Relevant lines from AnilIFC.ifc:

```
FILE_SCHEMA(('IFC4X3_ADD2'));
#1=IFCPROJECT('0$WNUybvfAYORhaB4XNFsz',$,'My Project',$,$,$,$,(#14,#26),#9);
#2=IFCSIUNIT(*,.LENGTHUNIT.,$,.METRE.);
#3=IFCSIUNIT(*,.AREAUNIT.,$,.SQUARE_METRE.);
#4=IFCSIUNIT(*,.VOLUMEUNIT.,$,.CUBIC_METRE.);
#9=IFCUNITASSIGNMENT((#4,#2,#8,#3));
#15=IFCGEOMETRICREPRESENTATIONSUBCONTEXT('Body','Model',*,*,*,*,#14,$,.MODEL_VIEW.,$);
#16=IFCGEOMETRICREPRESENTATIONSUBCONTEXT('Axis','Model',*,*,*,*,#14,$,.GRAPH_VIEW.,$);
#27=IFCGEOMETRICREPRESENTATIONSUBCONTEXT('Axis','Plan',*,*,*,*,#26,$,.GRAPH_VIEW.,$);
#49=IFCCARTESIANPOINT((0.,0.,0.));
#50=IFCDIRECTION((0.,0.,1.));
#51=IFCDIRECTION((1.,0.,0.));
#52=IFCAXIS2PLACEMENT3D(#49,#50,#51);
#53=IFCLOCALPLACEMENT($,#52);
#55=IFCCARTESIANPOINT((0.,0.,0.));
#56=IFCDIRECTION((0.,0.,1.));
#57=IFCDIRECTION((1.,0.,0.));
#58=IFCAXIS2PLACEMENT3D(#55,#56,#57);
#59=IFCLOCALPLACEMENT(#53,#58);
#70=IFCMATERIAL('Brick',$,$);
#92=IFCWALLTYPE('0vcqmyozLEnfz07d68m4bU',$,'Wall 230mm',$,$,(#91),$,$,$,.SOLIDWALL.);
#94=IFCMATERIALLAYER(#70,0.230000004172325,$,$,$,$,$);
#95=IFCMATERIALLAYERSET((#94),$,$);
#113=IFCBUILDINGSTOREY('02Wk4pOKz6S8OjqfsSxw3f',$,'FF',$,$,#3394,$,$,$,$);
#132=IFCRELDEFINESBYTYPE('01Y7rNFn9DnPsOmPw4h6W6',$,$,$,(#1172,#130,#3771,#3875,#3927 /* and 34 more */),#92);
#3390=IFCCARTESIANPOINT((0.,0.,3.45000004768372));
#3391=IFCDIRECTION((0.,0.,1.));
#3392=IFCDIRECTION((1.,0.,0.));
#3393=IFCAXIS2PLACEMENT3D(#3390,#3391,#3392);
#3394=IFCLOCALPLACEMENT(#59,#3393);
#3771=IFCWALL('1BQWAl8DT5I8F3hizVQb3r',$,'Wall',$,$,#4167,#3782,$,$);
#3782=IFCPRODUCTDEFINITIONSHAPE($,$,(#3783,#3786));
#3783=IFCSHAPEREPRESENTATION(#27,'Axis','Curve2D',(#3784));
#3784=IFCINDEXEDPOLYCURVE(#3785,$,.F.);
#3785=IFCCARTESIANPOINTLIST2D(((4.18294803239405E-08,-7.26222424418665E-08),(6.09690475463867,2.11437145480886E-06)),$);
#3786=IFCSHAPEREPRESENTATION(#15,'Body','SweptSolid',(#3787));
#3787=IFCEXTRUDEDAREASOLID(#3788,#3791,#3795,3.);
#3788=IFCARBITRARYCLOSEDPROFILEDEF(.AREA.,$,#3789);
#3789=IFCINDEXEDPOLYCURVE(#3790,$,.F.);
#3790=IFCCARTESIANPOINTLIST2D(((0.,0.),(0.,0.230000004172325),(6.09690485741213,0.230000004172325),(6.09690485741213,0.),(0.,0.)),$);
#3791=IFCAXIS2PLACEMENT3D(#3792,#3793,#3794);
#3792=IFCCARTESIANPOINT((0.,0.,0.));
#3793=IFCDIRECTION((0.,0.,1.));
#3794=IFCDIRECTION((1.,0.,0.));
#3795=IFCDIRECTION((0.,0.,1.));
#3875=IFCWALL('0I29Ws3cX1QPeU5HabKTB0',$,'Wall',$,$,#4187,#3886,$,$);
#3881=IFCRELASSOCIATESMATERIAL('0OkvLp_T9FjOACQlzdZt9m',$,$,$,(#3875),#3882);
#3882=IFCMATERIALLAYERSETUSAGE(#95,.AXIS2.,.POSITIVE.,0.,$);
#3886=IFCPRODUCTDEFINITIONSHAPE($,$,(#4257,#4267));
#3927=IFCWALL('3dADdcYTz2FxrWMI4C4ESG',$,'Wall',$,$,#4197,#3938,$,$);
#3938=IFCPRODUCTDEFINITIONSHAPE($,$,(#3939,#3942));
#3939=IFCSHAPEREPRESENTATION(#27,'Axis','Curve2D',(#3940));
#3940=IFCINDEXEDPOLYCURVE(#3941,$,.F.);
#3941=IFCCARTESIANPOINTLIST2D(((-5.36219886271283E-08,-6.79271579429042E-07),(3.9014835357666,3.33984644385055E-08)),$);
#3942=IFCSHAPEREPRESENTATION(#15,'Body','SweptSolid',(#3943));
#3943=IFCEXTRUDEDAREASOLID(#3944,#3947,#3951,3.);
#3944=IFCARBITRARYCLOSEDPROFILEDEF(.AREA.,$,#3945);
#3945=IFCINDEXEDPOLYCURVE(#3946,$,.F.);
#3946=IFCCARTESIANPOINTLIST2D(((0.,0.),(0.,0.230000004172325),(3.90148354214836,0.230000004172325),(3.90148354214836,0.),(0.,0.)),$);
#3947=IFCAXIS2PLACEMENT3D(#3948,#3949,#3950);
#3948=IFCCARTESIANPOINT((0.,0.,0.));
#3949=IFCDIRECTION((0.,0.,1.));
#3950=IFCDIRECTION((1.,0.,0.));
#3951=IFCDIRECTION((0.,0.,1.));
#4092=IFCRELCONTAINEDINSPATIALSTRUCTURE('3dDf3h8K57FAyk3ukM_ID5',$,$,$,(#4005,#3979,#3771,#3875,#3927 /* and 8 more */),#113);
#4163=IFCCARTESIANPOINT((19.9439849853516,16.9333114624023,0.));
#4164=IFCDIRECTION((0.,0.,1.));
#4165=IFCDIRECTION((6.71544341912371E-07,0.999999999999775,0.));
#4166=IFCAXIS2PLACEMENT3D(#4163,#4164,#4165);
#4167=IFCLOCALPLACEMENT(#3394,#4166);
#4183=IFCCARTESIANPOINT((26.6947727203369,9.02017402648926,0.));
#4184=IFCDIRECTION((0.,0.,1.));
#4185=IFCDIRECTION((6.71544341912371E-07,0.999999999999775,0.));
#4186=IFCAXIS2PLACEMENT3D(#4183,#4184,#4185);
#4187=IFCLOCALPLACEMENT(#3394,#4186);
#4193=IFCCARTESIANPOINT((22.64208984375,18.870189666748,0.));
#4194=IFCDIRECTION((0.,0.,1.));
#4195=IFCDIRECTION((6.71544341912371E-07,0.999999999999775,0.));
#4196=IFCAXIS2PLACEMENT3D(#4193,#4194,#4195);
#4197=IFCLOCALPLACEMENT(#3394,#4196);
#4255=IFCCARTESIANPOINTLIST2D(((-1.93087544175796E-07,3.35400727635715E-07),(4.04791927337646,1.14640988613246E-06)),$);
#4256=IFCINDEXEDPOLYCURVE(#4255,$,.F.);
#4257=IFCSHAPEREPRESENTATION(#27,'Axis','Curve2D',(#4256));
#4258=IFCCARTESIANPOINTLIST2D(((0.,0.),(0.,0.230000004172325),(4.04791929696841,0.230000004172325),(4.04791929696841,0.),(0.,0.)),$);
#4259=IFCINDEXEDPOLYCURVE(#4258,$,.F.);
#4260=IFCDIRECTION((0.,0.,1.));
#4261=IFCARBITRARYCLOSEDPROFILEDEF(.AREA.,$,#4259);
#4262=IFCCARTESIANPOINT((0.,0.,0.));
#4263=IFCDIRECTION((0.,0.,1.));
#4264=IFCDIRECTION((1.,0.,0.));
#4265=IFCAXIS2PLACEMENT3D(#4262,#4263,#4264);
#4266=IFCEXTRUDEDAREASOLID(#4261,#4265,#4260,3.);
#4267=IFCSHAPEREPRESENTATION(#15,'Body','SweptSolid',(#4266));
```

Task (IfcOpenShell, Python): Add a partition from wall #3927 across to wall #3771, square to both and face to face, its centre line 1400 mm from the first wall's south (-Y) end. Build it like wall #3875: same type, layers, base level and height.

```python
import numpy as np
import ifcopenshell
import ifcopenshell.api.geometry
import ifcopenshell.api.material
import ifcopenshell.api.pset
import ifcopenshell.api.root
import ifcopenshell.api.spatial
import ifcopenshell.api.type
import ifcopenshell.geom
import ifcopenshell.util.element
import ifcopenshell.util.placement
import ifcopenshell.util.representation
import ifcopenshell.util.shape
import ifcopenshell.util.unit

model = ifcopenshell.open("AnilIFC.ifc")
unit_scale = ifcopenshell.util.unit.calculate_unit_scale(model)
settings = ifcopenshell.geom.settings()
settings.set("use-world-coords", True)

start_wall = model.by_guid("3dADdcYTz2FxrWMI4C4ESG")
end_wall = model.by_guid("1BQWAl8DT5I8F3hizVQb3r")
like = model.by_id(3875)
matrix = ifcopenshell.util.placement.get_local_placement(start_wall.ObjectPlacement)
matrix[:3, 3] *= unit_scale


def extent(element):
    """Bounding box in the first wall's axes, in metres."""
    shape = ifcopenshell.geom.create_shape(settings, element)
    points = (ifcopenshell.util.shape.get_vertices(shape.geometry) - matrix[:3, 3]) @ matrix[:3, :3]
    return points.min(axis=0), points.max(axis=0)


y_start = extent(start_wall)[1][1]
y_end = extent(end_wall)[0][1]
like_min, like_max = extent(like)
length, height = float(abs(y_end - y_start)), float(like_max[2] - like_min[2])
layer_set = ifcopenshell.util.element.get_material(like, should_skip_usage=True)
thickness = sum(layer.LayerThickness for layer in layer_set.MaterialLayers) * unit_scale

wall = ifcopenshell.api.root.create_entity(model, ifc_class="IfcWall", name="New partition")
storey = ifcopenshell.util.element.get_container(like)
ifcopenshell.api.spatial.assign_container(model, products=[wall], relating_structure=storey)
ifcopenshell.api.type.assign_type(
    model, related_objects=[wall], relating_type=ifcopenshell.util.element.get_type(like), should_map_representations=False
)
rel = ifcopenshell.api.material.assign_material(
    model, products=[wall], type="IfcMaterialLayerSetUsage", material=layer_set
)
rel.RelatingMaterial.OffsetFromReferenceLine = -thickness / 2 / unit_scale
pset = ifcopenshell.api.pset.add_pset(model, product=wall, name="Pset_WallCommon")
ifcopenshell.api.pset.edit_pset(model, pset=pset, properties={"IsExternal": False, "LoadBearing": False})

# The axis runs down the middle of the wall.
axis = ifcopenshell.api.geometry.add_axis_representation(
    model, context=ifcopenshell.util.representation.get_context(model, "Model", "Axis"), axis=[(0.0, 0.0), (length, 0.0)]
)
body = ifcopenshell.api.geometry.add_wall_representation(
    model,
    context=ifcopenshell.util.representation.get_context(model, "Model", "Body", "MODEL_VIEW"),
    length=length,
    height=height,
    thickness=thickness,
    offset=-thickness / 2,
)
for representation in (axis, body):
    ifcopenshell.api.geometry.assign_representation(model, product=wall, representation=representation)

placement = matrix @ ifcopenshell.util.placement.rotation(90, "Z")
placement[:, 3] = matrix @ np.array([extent(start_wall)[0][0] + 1.4, y_start, like_min[2], 1.0])
ifcopenshell.api.geometry.edit_object_placement(model, product=wall, matrix=placement)

print(f"partition {length:.3f} m long, {height:.3f} m high, {thickness:.3f} m thick")

model.write("AnilIFC_rev.ifc")
```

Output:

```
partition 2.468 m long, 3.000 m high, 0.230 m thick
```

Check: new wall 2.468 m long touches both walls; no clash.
